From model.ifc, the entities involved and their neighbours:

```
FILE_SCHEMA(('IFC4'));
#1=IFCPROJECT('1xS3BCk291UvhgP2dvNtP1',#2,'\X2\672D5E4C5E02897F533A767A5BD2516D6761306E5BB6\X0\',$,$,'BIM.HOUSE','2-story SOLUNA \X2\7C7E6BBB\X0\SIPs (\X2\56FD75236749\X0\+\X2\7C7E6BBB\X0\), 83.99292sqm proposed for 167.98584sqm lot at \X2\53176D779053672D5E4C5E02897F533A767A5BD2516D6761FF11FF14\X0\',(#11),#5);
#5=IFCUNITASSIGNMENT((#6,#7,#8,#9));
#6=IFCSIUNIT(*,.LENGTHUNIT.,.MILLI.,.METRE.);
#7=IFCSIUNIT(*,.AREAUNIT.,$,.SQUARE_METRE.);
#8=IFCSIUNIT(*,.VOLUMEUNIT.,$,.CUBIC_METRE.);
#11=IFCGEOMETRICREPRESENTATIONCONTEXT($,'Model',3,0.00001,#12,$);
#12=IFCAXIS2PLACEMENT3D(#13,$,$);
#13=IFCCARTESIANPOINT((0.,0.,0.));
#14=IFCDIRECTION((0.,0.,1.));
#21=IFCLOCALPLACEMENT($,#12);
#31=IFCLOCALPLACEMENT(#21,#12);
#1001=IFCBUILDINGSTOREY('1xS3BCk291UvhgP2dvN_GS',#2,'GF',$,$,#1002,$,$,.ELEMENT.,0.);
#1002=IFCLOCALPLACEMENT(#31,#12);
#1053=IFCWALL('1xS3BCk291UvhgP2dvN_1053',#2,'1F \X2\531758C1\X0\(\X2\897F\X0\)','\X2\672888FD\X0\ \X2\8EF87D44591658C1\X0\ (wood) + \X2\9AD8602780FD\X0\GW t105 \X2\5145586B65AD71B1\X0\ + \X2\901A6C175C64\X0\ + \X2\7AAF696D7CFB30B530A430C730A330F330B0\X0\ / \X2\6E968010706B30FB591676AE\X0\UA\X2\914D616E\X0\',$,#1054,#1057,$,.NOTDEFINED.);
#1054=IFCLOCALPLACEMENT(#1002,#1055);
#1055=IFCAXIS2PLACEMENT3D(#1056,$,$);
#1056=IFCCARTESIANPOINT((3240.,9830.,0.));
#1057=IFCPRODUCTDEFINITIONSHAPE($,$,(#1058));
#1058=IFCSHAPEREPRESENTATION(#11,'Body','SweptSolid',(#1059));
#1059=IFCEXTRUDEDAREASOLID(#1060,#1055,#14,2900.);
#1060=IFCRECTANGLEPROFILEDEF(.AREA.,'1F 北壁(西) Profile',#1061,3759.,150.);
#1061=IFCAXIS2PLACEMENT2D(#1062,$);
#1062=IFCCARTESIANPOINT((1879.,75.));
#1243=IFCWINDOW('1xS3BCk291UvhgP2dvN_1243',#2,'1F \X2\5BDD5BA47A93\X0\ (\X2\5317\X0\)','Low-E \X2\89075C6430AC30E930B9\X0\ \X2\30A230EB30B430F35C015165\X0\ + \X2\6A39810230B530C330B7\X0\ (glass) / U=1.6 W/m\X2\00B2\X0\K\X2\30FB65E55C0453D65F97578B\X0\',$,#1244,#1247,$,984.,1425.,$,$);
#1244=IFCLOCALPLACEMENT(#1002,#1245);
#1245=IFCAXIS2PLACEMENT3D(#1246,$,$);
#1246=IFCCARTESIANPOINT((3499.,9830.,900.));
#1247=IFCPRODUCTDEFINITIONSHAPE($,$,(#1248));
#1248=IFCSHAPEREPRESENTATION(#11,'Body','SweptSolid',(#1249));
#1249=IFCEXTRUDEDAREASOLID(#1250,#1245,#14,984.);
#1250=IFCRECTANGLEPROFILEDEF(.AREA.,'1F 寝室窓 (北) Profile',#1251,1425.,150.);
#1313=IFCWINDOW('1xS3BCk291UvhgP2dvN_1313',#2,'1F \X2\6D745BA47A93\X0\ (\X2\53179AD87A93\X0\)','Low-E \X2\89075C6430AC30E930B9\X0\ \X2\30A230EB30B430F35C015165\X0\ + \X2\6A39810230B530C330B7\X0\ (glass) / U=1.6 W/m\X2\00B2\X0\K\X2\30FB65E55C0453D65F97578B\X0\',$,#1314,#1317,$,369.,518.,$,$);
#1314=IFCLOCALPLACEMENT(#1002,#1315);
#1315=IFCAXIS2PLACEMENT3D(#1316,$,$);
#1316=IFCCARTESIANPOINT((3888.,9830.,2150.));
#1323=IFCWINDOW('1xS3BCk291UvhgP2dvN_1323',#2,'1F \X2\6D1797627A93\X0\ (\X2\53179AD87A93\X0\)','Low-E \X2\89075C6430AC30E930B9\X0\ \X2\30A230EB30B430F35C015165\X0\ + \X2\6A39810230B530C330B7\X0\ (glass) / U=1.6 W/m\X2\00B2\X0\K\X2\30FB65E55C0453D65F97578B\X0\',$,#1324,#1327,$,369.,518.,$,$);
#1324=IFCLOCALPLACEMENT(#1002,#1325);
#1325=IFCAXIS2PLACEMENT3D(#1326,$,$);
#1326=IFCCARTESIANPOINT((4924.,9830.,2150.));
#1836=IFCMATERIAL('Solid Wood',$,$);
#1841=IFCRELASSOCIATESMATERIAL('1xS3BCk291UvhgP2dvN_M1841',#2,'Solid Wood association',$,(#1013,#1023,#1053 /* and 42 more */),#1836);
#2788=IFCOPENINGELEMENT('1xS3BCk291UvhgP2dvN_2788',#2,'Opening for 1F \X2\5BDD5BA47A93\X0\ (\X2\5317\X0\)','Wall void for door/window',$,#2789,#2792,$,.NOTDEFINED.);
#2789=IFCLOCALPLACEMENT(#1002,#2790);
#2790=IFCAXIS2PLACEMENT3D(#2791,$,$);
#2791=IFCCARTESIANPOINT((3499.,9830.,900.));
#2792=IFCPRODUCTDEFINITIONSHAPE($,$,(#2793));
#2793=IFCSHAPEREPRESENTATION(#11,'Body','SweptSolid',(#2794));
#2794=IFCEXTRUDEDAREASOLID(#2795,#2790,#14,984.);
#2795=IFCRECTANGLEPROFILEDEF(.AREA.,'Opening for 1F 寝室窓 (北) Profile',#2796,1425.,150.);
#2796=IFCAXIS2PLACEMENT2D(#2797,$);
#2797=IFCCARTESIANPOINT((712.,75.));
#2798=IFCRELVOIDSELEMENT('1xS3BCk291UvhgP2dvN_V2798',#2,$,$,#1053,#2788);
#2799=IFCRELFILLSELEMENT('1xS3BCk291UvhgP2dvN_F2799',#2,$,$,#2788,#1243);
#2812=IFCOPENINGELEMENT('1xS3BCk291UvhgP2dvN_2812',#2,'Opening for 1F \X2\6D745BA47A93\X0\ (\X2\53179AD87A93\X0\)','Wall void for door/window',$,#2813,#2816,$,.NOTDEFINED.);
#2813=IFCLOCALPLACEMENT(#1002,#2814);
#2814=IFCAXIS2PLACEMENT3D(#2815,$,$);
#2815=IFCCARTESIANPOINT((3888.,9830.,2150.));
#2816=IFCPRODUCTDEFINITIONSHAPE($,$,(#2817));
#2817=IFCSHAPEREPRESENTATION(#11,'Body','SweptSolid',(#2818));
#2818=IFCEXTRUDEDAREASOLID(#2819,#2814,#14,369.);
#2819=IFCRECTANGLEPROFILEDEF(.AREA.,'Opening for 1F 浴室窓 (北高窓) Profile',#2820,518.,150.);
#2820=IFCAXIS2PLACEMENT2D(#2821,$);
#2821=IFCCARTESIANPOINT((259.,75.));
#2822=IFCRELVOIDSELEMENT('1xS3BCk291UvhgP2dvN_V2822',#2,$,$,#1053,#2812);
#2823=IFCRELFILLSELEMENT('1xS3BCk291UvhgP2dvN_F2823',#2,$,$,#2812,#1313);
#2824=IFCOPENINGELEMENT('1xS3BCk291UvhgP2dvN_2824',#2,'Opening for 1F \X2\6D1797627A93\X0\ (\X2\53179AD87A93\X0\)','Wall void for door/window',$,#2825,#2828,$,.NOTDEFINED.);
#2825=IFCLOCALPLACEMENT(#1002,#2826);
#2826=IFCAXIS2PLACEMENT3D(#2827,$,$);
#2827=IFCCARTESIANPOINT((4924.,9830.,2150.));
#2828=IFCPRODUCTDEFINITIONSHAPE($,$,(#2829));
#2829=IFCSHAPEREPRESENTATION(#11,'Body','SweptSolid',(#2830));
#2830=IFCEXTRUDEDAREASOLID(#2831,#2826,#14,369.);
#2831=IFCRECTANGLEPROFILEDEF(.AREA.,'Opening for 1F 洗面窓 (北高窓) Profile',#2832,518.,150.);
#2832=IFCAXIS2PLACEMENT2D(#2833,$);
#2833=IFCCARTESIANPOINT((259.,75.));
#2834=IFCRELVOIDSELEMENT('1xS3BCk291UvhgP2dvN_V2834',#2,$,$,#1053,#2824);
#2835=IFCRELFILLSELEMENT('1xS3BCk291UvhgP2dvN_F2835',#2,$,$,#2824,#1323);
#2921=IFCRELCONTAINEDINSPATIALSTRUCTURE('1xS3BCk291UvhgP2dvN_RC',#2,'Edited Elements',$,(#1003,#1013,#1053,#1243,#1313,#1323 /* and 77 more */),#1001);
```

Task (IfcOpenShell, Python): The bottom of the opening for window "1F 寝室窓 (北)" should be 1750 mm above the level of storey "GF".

```python
import numpy as np
import ifcopenshell
import ifcopenshell.api.geometry
import ifcopenshell.geom
import ifcopenshell.util.element
import ifcopenshell.util.placement
import ifcopenshell.util.shape
import ifcopenshell.util.unit

model = ifcopenshell.open("model.ifc")
unit_scale = ifcopenshell.util.unit.calculate_unit_scale(model)

window = model.by_guid("1xS3BCk291UvhgP2dvN_1243")
opening = window.FillsVoids[0].RelatingOpeningElement
storey = ifcopenshell.util.element.get_container(window, ifc_class="IfcBuildingStorey")
level = ifcopenshell.util.placement.get_local_placement(storey.ObjectPlacement)[2, 3]

# The opening's origin need not be at the sill, so measure its lowest point.
shape = ifcopenshell.geom.create_shape(ifcopenshell.geom.settings(), opening)
bottom = ifcopenshell.util.shape.get_shape_bottom_elevation(shape, shape.geometry) / unit_scale
dz = level + 1.75 / unit_scale - bottom

shift = np.array([0.0, 0.0, dz])
# The window is not placed relative to its opening, so move both.
for product in (opening, window):
    matrix = ifcopenshell.util.placement.get_local_placement(product.ObjectPlacement)
    matrix[:3, 3] += shift
    ifcopenshell.api.geometry.edit_object_placement(model, product=product, matrix=matrix, is_si=False)

print(f"moved by {dz * unit_scale:+.3f} m")

model.write("model_rev.ifc")
```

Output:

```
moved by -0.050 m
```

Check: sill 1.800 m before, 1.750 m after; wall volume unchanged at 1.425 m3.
